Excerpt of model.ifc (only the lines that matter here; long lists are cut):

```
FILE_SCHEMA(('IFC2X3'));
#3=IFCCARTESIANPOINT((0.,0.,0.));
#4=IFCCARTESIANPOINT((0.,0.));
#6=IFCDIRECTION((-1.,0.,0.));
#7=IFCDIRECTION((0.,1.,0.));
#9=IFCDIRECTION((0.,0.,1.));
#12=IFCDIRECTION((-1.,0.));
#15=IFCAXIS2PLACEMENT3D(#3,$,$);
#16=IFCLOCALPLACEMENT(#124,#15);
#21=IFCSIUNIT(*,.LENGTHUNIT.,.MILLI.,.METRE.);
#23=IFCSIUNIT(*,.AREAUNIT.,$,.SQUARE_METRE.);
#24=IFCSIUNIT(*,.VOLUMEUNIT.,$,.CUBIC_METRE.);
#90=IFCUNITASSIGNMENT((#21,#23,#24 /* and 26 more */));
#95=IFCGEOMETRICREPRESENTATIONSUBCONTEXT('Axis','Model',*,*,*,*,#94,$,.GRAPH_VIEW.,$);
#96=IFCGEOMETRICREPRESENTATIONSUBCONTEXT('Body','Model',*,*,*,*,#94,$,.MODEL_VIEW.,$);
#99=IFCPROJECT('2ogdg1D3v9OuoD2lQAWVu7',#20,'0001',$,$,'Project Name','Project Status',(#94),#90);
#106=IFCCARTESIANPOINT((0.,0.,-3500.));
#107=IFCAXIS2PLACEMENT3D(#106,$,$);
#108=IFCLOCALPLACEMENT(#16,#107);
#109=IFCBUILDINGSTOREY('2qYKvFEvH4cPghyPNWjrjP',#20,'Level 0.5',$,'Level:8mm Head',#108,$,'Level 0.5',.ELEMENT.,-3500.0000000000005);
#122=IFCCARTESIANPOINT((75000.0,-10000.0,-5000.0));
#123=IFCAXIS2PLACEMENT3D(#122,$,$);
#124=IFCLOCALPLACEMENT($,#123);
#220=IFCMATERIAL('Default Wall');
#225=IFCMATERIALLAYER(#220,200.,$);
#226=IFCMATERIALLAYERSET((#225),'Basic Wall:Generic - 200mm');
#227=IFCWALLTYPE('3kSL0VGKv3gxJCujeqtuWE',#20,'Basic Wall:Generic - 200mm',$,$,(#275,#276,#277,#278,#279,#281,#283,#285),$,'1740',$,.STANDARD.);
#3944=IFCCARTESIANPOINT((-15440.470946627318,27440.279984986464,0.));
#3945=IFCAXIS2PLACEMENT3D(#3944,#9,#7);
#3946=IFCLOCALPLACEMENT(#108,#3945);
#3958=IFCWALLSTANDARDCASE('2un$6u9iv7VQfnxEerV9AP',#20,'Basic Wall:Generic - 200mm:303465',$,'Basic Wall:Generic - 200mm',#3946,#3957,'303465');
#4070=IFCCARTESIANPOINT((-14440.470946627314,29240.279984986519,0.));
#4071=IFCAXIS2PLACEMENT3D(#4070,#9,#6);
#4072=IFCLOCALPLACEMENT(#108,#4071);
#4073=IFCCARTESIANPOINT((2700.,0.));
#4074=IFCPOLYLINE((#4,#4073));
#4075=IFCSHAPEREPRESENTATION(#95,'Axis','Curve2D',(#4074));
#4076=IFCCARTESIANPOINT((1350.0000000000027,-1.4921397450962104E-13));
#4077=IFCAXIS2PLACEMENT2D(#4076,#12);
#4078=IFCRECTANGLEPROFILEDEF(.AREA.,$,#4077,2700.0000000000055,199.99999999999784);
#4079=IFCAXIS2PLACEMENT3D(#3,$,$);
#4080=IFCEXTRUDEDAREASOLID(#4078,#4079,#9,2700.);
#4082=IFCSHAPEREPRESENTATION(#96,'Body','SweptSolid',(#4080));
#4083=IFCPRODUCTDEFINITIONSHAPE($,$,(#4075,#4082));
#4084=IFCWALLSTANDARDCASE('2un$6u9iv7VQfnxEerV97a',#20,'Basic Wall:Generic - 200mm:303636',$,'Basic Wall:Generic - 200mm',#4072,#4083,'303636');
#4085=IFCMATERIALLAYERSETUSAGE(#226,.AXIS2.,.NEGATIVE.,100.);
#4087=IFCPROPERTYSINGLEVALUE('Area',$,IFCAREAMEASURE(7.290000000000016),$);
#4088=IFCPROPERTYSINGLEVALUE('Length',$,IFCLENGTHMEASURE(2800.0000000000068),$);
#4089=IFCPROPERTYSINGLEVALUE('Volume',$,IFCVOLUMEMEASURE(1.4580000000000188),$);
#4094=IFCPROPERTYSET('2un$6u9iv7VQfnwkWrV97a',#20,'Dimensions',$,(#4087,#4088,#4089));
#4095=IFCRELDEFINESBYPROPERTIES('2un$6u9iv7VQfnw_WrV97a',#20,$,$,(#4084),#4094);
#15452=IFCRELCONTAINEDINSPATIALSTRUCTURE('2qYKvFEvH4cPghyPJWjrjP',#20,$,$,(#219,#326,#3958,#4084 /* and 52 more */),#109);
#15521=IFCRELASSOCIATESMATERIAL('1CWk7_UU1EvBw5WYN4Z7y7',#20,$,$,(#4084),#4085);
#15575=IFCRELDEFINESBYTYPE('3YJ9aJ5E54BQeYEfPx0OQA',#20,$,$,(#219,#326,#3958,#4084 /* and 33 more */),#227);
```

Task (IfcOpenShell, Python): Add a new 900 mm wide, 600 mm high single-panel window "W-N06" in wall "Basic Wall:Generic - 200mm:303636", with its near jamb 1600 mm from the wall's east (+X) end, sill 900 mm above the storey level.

```python
import numpy as np
import ifcopenshell
import ifcopenshell.api.feature
import ifcopenshell.api.geometry
import ifcopenshell.api.pset
import ifcopenshell.api.root
import ifcopenshell.api.spatial
import ifcopenshell.api.type
import ifcopenshell.geom
import ifcopenshell.util.element
import ifcopenshell.util.placement
import ifcopenshell.util.representation
import ifcopenshell.util.shape
import ifcopenshell.util.unit

model = ifcopenshell.open("model.ifc")
unit_scale = ifcopenshell.util.unit.calculate_unit_scale(model)
area_scale = ifcopenshell.util.unit.calculate_unit_scale(model, "AREAUNIT")
volume_scale = ifcopenshell.util.unit.calculate_unit_scale(model, "VOLUMEUNIT")
settings = ifcopenshell.geom.settings()


def volume(element):
    """Net volume in cubic metres, openings subtracted."""
    shape = ifcopenshell.geom.create_shape(settings, element)
    return ifcopenshell.util.shape.get_volume(shape.geometry)


wall = model.by_id(4084)
storey = ifcopenshell.util.element.get_container(wall, ifc_class="IfcBuildingStorey")
context = ifcopenshell.util.representation.get_context(model, "Model", "Body", "MODEL_VIEW")
before = volume(wall)

width, height, from_end, sill = 0.9, 0.6, 1.6, 0.9  # metres

# The wall runs along its own X axis, and the end named is its -X end.
wall_shape = ifcopenshell.geom.create_shape(settings, wall)
x, y, z = ifcopenshell.util.shape.get_vertices(wall_shape.geometry).T
start = x.min() + from_end
face, thickness = float(y.min()), float(y.max() - y.min())
wall_matrix = ifcopenshell.util.placement.get_local_placement(wall.ObjectPlacement)
level = ifcopenshell.util.placement.get_local_placement(storey.ObjectPlacement)[2, 3]


def in_wall(x, y):
    """Placement at x, y metres in the wall's axes, at sill height."""
    matrix = wall_matrix.copy()
    matrix[:, 3] = wall_matrix @ np.array([x / unit_scale, y / unit_scale, 0.0, 1.0])
    matrix[2, 3] = level + sill / unit_scale
    return matrix


# Opening: a box that overshoots both wall faces by 50 mm.
opening = ifcopenshell.api.root.create_entity(model, ifc_class="IfcOpeningElement")
box = ifcopenshell.api.geometry.add_wall_representation(
    model, context=context, length=width, height=height, thickness=thickness + 0.1
)
ifcopenshell.api.geometry.assign_representation(model, product=opening, representation=box)
ifcopenshell.api.geometry.edit_object_placement(model, product=opening, matrix=in_wall(start, face - 0.05), is_si=False)
ifcopenshell.api.feature.add_feature(model, feature=opening, element=wall)

window = ifcopenshell.api.root.create_entity(model, ifc_class="IfcWindow", name="W-N06")
window.OverallWidth, window.OverallHeight = width / unit_scale, height / unit_scale
body = ifcopenshell.api.geometry.add_window_representation(
    model,
    context=context,
    overall_width=window.OverallWidth,
    overall_height=window.OverallHeight,
    partition_type="SINGLE_PANEL",
)
ifcopenshell.api.geometry.assign_representation(model, product=window, representation=body)
ifcopenshell.api.spatial.assign_container(model, products=[window], relating_structure=storey)
fills = ifcopenshell.api.feature.add_filling(model, opening=opening, element=window)
fills.OwnerHistory = window.OwnerHistory  # required in IFC2X3

# IFC2X3 keeps the operation on the window style.
style = ifcopenshell.api.root.create_entity(model, ifc_class="IfcWindowStyle", name="W-N06")
style.OperationType, style.ConstructionType = "SINGLE_PANEL", "NOTDEFINED"
style.ParameterTakesPrecedence = style.Sizeable = False
ifcopenshell.api.type.assign_type(model, related_objects=[window], relating_type=style)

# Centre the window in the wall's thickness.
ifcopenshell.api.geometry.edit_object_placement(model, product=window, matrix=in_wall(start, face), is_si=False)
window_shape = ifcopenshell.geom.create_shape(settings, window)
depth = ifcopenshell.util.shape.get_vertices(window_shape.geometry)[:, 1]
offset = face + thickness / 2 - (depth.min() + depth.max()) / 2
ifcopenshell.api.geometry.edit_object_placement(model, product=window, matrix=in_wall(start, offset), is_si=False)

after = volume(wall)

# Update the wall's stored quantities.
pset = model.by_id(ifcopenshell.util.element.get_pset(wall, "Dimensions", should_inherit=False)["id"])
ifcopenshell.api.pset.edit_pset(model, pset=pset, properties={
    "Area": model.create_entity("IfcAreaMeasure", after / thickness / area_scale),
    "Volume": model.create_entity("IfcVolumeMeasure", after / volume_scale),
})

print(f"wall volume {before:.3f} -> {after:.3f} m3")

model.write("model_rev.ifc")
```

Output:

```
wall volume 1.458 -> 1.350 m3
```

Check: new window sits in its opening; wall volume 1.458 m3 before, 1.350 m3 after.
